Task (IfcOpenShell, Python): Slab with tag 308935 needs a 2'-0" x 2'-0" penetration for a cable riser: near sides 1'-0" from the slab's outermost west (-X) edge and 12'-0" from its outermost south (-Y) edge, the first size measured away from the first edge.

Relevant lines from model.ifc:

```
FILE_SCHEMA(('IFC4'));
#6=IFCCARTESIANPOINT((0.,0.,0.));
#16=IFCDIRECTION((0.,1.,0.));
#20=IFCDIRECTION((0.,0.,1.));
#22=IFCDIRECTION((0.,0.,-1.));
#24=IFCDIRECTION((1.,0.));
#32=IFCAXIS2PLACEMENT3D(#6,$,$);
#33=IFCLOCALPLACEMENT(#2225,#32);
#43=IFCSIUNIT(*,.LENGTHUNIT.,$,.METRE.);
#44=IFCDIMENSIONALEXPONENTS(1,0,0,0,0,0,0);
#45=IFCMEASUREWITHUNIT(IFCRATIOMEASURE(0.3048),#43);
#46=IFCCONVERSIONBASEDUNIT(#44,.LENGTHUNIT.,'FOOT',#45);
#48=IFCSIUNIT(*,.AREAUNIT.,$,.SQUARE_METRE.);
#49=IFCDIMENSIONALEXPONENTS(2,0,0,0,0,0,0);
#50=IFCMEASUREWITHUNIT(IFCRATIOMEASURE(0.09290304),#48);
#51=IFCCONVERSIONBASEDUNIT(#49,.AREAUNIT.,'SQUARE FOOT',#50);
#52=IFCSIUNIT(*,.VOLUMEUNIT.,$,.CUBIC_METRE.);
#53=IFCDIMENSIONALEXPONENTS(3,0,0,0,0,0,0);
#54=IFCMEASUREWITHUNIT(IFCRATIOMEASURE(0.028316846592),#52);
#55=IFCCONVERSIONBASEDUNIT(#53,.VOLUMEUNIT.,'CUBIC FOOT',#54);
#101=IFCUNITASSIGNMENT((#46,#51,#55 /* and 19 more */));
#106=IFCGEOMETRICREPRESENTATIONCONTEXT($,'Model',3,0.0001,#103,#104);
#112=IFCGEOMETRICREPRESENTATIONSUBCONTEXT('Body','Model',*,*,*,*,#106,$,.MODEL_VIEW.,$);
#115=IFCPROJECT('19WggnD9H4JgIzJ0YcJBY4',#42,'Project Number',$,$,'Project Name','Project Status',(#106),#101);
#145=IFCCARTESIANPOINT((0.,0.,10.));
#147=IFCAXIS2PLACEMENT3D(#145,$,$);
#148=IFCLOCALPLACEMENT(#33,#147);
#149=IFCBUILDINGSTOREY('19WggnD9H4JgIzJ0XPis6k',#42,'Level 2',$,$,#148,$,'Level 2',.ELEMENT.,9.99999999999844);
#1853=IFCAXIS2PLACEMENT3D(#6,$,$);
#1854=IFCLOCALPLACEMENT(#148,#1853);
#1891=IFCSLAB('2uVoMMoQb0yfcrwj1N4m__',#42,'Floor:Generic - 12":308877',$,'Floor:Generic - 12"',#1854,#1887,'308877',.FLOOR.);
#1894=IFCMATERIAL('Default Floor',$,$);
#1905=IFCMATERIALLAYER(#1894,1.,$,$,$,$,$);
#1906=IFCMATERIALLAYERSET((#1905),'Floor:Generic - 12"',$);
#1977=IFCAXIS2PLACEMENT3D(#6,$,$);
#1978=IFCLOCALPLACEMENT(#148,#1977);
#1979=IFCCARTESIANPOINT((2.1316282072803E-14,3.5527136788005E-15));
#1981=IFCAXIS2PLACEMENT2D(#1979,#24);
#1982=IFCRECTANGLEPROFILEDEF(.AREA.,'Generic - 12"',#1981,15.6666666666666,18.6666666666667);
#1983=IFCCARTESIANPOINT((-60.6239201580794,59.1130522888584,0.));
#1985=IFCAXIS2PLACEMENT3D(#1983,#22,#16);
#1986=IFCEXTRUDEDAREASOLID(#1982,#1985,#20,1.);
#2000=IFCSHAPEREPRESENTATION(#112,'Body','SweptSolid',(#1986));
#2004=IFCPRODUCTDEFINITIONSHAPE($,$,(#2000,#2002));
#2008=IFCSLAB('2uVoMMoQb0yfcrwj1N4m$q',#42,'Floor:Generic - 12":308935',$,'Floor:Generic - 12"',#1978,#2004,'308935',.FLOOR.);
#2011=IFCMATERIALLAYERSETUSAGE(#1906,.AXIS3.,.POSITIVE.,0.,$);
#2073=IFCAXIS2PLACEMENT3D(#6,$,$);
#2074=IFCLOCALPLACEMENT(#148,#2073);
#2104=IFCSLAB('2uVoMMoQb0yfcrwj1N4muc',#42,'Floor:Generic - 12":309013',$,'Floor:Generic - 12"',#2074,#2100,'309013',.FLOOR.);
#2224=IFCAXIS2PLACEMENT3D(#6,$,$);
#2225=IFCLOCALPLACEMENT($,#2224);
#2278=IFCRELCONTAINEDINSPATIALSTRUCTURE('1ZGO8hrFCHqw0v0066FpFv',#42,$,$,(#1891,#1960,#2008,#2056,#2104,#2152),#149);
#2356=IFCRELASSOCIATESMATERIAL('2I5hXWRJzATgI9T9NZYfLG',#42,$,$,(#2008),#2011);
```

```python
import numpy as np
import ifcopenshell
import ifcopenshell.api.feature
import ifcopenshell.api.geometry
import ifcopenshell.api.root
import ifcopenshell.geom
import ifcopenshell.util.placement
import ifcopenshell.util.representation
import ifcopenshell.util.shape
import ifcopenshell.util.unit

model = ifcopenshell.open("model.ifc")
unit_scale = ifcopenshell.util.unit.calculate_unit_scale(model)
settings = ifcopenshell.geom.settings()


def volume(element):
    """Net volume in cubic metres, openings subtracted."""
    shape = ifcopenshell.geom.create_shape(settings, element)
    return ifcopenshell.util.shape.get_volume(shape.geometry)


slab = model.by_guid("2uVoMMoQb0yfcrwj1N4m$q")
before = volume(slab)

# Extent in the slab's own axes, in metres. The edges named are its -X and -Y sides.
slab_shape = ifcopenshell.geom.create_shape(settings, slab)
vertices = ifcopenshell.util.shape.get_vertices(slab_shape.geometry)
x_min, y_min, bottom = vertices.min(axis=0)
top = vertices[:, 2].max()

opening = ifcopenshell.api.root.create_entity(model, ifc_class="IfcOpeningElement", name="Cable riser opening", predefined_type="OPENING")
context = ifcopenshell.util.representation.get_context(model, "Model", "Body", "MODEL_VIEW")
width, depth = 0.6096, 0.6096
outline = [(0.0, 0.0), (width, 0.0), (width, depth), (0.0, depth), (0.0, 0.0)]
# Overshoot both faces by 50 mm so the cut is clean.
shape = ifcopenshell.api.geometry.add_slab_representation(
    model, context=context, depth=top - bottom + 0.1, polyline=outline
)
ifcopenshell.api.geometry.assign_representation(model, product=opening, representation=shape)

matrix = ifcopenshell.util.placement.get_local_placement(slab.ObjectPlacement)
matrix[:, 3] = matrix @ np.append(np.array([x_min + 0.3048, y_min + 3.6576, bottom - 0.05]) / unit_scale, 1.0)
ifcopenshell.api.geometry.edit_object_placement(model, product=opening, matrix=matrix, is_si=False)
ifcopenshell.api.feature.add_feature(model, feature=opening, element=slab)

after = volume(slab)

print(f"slab volume {before:.3f} -> {after:.3f} m3")

model.write("model-out.ifc")
```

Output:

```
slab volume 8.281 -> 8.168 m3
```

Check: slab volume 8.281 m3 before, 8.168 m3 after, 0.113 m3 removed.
